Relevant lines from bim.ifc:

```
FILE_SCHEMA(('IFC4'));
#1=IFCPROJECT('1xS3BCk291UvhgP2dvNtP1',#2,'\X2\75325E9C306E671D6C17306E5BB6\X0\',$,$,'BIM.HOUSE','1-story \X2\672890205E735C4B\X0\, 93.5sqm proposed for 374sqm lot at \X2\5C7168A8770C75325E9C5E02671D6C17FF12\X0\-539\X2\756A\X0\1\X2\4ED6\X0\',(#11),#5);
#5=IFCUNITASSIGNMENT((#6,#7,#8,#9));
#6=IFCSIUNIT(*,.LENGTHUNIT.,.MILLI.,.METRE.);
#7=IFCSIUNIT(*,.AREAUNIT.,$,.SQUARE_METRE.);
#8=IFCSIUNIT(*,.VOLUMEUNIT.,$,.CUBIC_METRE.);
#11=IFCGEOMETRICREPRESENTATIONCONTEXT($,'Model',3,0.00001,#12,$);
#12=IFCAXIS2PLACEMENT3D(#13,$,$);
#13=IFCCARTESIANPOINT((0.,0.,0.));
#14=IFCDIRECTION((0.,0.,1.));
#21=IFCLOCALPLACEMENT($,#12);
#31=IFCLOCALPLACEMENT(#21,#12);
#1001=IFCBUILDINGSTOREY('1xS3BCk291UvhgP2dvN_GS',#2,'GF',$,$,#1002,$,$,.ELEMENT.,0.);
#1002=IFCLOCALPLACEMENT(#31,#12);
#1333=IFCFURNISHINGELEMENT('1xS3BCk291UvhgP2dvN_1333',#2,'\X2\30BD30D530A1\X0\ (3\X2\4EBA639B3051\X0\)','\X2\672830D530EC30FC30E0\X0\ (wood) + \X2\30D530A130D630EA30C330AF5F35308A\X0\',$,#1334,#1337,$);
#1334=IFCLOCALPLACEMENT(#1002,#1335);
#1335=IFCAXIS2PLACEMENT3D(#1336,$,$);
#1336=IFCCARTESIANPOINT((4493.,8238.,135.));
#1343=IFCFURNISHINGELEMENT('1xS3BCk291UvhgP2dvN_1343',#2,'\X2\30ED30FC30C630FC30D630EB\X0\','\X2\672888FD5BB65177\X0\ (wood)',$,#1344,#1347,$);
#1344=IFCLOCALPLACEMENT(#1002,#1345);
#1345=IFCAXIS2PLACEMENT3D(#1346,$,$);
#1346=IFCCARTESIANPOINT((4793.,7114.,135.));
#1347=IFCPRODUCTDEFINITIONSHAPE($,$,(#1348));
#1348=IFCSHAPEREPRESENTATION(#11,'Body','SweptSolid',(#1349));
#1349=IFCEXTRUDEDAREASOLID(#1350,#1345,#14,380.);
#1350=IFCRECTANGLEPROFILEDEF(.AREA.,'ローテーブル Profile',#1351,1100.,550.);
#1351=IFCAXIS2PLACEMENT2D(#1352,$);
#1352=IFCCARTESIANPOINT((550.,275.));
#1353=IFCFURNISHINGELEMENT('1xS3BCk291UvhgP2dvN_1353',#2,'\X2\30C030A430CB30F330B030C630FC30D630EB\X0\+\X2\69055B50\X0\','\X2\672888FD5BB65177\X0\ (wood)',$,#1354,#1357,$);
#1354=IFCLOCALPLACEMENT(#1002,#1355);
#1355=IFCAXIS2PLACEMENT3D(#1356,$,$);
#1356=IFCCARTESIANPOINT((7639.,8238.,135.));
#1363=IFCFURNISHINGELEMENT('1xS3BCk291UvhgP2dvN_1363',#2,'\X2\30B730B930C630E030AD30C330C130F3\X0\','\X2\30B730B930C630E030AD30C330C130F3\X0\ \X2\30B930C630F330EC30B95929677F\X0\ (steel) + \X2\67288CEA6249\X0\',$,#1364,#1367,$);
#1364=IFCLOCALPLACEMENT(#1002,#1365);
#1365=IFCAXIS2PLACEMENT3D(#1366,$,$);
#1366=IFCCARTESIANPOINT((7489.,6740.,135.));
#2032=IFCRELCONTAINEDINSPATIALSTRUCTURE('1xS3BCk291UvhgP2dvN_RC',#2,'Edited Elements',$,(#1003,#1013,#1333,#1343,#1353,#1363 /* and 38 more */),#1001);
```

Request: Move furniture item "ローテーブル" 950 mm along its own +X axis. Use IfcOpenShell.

```python
import ifcopenshell
import ifcopenshell.api.geometry
import ifcopenshell.util.placement

model = ifcopenshell.open("bim.ifc")

item = model.by_guid("1xS3BCk291UvhgP2dvN_1343")
matrix = ifcopenshell.util.placement.get_local_placement(item.ObjectPlacement)
matrix[:3, 3] += matrix[:3, 0] * 950.0
ifcopenshell.api.geometry.edit_object_placement(model, product=item, matrix=matrix, is_si=False)

print(ifcopenshell.util.placement.get_local_placement(item.ObjectPlacement).round(3) + 0.0)

model.write("bim_updated.ifc")
```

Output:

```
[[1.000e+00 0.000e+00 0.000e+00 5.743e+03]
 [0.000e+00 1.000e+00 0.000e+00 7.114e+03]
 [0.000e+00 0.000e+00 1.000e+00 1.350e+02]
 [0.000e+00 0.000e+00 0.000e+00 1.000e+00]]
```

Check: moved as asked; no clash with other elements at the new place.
